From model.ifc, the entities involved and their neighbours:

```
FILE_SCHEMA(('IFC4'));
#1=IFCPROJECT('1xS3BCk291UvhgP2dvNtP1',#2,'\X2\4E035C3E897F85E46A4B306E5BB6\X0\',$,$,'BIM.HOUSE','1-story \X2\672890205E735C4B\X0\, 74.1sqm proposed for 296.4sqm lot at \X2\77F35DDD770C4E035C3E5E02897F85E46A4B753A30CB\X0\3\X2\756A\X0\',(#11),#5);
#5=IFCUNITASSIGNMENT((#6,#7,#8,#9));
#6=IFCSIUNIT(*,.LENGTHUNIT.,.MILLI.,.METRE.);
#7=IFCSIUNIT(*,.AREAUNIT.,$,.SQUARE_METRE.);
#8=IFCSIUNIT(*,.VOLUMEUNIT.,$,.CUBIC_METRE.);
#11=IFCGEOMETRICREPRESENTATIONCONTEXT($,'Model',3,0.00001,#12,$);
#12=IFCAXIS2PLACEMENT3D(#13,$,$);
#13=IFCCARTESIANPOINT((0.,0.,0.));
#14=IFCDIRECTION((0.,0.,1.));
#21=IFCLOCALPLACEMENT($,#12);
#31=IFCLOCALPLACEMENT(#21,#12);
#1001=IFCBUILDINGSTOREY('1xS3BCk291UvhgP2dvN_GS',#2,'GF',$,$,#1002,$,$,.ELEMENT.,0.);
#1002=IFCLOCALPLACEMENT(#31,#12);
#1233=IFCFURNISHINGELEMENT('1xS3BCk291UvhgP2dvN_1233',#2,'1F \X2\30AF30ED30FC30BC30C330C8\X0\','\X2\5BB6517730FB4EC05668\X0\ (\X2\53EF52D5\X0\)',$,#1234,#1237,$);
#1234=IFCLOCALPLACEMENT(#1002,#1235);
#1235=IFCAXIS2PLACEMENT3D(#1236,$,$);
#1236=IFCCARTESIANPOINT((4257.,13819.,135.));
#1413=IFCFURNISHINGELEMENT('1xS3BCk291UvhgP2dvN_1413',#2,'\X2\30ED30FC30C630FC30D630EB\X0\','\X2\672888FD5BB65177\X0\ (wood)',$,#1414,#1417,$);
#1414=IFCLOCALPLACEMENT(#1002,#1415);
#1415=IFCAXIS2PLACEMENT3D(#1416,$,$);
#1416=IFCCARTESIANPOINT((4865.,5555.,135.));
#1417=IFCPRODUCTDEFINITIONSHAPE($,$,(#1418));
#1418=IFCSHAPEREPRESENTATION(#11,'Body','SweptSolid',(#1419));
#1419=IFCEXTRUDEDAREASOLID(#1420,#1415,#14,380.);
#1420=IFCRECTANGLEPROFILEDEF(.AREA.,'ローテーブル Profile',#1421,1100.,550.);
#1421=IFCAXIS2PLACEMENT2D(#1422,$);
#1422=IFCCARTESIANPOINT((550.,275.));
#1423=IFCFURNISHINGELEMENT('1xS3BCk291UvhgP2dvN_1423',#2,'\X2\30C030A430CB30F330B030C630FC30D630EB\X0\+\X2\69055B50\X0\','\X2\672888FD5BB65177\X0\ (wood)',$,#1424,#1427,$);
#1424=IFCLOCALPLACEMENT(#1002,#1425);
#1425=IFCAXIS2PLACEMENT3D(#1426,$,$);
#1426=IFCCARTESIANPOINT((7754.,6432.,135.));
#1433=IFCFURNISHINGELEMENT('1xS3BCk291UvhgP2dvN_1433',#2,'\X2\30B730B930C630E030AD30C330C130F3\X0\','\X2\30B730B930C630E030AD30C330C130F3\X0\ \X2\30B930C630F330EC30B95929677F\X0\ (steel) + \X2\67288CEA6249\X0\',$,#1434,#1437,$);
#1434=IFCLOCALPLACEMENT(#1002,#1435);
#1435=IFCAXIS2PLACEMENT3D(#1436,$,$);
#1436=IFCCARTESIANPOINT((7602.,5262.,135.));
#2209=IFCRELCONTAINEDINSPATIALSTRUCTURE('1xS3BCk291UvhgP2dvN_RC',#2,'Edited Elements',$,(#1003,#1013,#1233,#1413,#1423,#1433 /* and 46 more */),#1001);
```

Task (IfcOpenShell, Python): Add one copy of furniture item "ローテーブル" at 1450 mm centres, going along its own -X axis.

```python
import ifcopenshell
import ifcopenshell.api.geometry
import ifcopenshell.api.root
import ifcopenshell.util.element
import ifcopenshell.util.placement

model = ifcopenshell.open("model.ifc")


def reuse_history(source, copy):
    """copy_class also copies each property set's owner history, people and application; keep the originals."""
    for rel in copy.IsDefinedBy:
        if rel.is_a("IfcRelDefinesByProperties") and (history := rel.RelatingPropertyDefinition.OwnerHistory):
            rel.RelatingPropertyDefinition.OwnerHistory = source.OwnerHistory
            ifcopenshell.util.element.remove_deep2(model, history)


source = model.by_guid("1xS3BCk291UvhgP2dvN_1413")
base = ifcopenshell.util.placement.get_local_placement(source.ObjectPlacement)
step = -base[:3, 0] * 1450.0

for i in range(1, 2):
    copy = ifcopenshell.api.root.copy_class(model, product=source)
    copy.Representation = ifcopenshell.util.element.copy_deep(
        model, source.Representation, exclude=["IfcGeometricRepresentationContext", "IfcRepresentationMap"]
    )
    reuse_history(source, copy)
    matrix = base.copy()
    matrix[:3, 3] += i * step
    print("added at", matrix[:3, 3].round(3) + 0.0)
    ifcopenshell.api.geometry.edit_object_placement(model, product=copy, matrix=matrix, is_si=False)

model.write("model_edited.ifc")
```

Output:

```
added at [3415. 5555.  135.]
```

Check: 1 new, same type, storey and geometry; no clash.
